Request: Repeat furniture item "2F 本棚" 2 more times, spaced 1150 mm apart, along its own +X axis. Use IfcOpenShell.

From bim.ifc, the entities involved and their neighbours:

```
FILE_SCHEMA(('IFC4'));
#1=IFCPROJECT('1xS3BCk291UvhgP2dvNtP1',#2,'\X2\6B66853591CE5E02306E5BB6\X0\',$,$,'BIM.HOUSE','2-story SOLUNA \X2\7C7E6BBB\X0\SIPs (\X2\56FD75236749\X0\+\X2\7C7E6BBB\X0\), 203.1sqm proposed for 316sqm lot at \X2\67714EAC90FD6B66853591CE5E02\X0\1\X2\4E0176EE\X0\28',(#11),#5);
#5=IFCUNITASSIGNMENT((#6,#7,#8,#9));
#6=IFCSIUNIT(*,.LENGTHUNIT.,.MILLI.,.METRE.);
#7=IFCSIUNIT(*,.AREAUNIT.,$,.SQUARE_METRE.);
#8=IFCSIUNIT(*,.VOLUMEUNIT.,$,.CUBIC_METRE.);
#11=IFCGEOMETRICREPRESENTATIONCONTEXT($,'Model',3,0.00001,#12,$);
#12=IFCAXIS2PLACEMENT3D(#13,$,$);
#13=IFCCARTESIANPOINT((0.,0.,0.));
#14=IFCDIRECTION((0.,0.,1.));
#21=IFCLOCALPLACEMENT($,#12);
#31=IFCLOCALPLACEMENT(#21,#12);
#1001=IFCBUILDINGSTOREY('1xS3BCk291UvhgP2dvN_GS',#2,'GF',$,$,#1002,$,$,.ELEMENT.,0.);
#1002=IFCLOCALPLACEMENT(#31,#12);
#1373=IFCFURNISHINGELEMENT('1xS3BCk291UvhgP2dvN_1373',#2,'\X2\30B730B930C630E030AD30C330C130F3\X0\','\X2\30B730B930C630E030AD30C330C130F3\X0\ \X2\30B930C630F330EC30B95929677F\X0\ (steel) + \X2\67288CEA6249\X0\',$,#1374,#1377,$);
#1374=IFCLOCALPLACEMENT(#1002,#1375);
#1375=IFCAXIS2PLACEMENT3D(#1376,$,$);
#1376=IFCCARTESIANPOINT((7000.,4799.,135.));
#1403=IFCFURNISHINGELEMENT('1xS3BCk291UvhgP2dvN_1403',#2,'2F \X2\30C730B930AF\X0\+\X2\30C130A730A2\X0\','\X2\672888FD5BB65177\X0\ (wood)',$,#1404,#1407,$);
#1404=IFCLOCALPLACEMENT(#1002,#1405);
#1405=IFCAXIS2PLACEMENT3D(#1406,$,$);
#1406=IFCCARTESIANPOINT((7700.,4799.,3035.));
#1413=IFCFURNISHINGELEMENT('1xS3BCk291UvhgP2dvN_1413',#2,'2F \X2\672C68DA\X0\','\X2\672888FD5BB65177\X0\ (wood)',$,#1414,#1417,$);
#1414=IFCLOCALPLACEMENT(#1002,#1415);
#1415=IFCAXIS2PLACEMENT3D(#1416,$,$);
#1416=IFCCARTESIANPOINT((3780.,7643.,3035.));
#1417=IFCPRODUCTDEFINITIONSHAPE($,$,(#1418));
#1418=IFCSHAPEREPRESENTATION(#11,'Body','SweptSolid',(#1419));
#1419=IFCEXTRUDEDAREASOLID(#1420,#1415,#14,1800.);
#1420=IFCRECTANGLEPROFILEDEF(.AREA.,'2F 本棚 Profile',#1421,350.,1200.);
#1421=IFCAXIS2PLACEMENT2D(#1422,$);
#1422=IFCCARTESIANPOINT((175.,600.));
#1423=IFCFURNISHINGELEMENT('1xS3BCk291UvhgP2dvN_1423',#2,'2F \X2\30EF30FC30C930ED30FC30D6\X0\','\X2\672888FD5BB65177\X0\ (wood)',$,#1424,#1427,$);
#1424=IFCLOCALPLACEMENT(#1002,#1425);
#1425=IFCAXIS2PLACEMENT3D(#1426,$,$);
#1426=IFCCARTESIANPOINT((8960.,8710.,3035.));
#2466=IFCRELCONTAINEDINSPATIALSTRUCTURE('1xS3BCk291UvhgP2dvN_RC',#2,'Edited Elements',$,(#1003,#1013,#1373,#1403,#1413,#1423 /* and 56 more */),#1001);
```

```python
import ifcopenshell
import ifcopenshell.api.geometry
import ifcopenshell.api.root
import ifcopenshell.util.element
import ifcopenshell.util.placement
import ifcopenshell.util.unit

model = ifcopenshell.open("bim.ifc")
unit_scale = ifcopenshell.util.unit.calculate_unit_scale(model)


def reuse_history(source, copy):
    """copy_class also copies each property set's owner history, people and application; keep the originals."""
    for rel in copy.IsDefinedBy:
        if rel.is_a("IfcRelDefinesByProperties") and (history := rel.RelatingPropertyDefinition.OwnerHistory):
            rel.RelatingPropertyDefinition.OwnerHistory = source.OwnerHistory
            ifcopenshell.util.element.remove_deep2(model, history)


source = model.by_guid("1xS3BCk291UvhgP2dvN_1413")
base = ifcopenshell.util.placement.get_local_placement(source.ObjectPlacement)
step = base[:3, 0] * 1.15 / unit_scale

for i in range(1, 3):
    copy = ifcopenshell.api.root.copy_class(model, product=source)
    copy.Representation = ifcopenshell.util.element.copy_deep(
        model, source.Representation, exclude=["IfcGeometricRepresentationContext", "IfcRepresentationMap"]
    )
    reuse_history(source, copy)
    matrix = base.copy()
    matrix[:3, 3] += i * step
    print("added at", matrix[:3, 3].round(3) + 0.0)
    ifcopenshell.api.geometry.edit_object_placement(model, product=copy, matrix=matrix, is_si=False)

model.write("bim_updated.ifc")
```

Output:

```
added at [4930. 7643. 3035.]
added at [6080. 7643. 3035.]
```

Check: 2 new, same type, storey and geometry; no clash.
